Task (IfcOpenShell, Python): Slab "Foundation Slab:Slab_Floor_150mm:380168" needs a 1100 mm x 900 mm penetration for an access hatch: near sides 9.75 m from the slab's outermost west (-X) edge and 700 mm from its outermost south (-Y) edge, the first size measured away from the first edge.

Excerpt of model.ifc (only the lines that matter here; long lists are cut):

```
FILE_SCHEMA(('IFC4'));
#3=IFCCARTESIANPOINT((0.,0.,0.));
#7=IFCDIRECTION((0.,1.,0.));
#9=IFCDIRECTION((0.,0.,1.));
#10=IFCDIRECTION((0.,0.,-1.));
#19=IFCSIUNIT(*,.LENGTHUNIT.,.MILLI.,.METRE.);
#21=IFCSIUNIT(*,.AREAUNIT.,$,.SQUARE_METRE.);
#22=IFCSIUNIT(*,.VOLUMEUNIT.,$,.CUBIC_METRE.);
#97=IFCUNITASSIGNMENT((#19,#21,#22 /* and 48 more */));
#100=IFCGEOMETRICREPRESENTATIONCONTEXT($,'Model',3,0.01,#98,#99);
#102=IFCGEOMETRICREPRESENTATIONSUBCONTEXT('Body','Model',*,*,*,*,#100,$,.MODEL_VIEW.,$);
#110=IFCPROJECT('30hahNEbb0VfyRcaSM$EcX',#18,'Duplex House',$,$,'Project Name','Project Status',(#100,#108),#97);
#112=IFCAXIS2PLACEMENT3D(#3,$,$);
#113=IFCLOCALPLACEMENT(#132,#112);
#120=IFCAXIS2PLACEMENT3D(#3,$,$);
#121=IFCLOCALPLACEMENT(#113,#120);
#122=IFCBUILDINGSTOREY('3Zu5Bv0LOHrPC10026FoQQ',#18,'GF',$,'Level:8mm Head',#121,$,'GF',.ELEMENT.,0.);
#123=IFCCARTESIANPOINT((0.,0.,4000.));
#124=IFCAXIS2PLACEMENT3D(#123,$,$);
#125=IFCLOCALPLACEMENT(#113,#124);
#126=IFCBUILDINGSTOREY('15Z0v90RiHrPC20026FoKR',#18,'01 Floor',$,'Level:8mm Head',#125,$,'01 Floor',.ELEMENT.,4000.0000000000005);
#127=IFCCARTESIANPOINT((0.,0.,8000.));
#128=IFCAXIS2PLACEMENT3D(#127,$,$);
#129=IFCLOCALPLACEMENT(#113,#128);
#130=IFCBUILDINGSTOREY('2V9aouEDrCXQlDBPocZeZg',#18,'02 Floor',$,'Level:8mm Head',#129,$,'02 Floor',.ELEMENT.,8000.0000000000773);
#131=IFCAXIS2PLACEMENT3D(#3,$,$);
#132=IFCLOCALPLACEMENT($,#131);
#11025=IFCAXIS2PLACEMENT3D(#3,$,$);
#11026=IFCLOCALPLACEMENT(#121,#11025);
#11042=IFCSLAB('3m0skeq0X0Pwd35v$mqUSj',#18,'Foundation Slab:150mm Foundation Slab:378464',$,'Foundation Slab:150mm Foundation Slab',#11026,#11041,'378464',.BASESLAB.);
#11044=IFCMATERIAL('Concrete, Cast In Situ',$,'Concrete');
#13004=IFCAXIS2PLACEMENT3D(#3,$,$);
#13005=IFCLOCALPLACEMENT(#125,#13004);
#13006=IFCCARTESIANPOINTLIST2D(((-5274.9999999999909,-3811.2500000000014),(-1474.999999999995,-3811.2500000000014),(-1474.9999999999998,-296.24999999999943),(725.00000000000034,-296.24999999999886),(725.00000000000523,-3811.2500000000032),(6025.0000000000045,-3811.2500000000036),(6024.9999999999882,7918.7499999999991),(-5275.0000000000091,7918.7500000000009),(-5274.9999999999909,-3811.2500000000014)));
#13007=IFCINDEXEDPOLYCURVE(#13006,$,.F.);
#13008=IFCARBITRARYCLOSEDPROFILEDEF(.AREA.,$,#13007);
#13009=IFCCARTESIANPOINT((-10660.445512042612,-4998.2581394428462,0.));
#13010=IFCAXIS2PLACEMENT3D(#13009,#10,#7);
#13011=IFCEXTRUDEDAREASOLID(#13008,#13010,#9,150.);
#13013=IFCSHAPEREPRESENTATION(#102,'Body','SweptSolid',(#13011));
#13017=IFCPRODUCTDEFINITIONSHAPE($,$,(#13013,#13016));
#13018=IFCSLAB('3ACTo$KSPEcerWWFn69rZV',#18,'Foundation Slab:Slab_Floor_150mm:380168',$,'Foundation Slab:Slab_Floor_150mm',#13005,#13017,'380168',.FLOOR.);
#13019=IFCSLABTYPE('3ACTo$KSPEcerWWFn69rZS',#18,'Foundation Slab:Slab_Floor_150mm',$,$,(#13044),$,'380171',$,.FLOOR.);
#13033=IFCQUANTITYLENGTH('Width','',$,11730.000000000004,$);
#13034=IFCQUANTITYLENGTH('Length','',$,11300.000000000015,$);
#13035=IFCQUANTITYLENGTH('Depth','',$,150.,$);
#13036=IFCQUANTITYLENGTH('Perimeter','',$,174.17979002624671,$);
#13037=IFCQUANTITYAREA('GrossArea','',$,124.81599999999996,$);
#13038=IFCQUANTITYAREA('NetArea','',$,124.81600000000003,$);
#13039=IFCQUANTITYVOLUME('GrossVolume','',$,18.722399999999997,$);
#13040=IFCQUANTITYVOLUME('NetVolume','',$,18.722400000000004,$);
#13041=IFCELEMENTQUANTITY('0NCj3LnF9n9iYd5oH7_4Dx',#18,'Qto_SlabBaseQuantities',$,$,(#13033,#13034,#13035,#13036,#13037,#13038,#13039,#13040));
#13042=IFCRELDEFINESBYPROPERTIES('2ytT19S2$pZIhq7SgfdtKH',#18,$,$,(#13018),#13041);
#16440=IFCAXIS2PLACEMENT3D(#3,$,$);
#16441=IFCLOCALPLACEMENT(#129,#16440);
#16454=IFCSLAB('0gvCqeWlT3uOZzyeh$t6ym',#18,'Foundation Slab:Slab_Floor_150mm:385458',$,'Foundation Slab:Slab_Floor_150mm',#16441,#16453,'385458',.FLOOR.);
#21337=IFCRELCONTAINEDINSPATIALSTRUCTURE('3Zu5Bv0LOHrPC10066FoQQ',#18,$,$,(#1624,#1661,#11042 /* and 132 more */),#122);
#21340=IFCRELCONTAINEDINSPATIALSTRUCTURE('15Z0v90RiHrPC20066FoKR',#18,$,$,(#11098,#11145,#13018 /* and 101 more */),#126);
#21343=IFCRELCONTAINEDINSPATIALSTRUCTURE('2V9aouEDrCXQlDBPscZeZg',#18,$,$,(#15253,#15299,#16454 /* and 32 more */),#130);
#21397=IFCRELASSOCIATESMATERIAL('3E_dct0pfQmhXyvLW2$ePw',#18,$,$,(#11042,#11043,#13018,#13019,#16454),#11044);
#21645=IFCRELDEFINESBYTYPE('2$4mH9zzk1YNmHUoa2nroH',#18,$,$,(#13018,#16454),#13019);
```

```python
import numpy as np
import ifcopenshell
import ifcopenshell.api.feature
import ifcopenshell.api.geometry
import ifcopenshell.api.pset
import ifcopenshell.api.root
import ifcopenshell.geom
import ifcopenshell.util.element
import ifcopenshell.util.placement
import ifcopenshell.util.representation
import ifcopenshell.util.shape
import ifcopenshell.util.unit

model = ifcopenshell.open("model.ifc")
unit_scale = ifcopenshell.util.unit.calculate_unit_scale(model)
area_scale = ifcopenshell.util.unit.calculate_unit_scale(model, "AREAUNIT")
volume_scale = ifcopenshell.util.unit.calculate_unit_scale(model, "VOLUMEUNIT")
settings = ifcopenshell.geom.settings()


def volume(element):
    """Net volume in cubic metres, openings subtracted."""
    shape = ifcopenshell.geom.create_shape(settings, element)
    return ifcopenshell.util.shape.get_volume(shape.geometry)


slab = model.by_id(13018)
before = volume(slab)

# Extent in the slab's own axes, in metres. The edges named are its -X and -Y sides.
slab_shape = ifcopenshell.geom.create_shape(settings, slab)
vertices = ifcopenshell.util.shape.get_vertices(slab_shape.geometry)
x_min, y_min, bottom = vertices.min(axis=0)
top = vertices[:, 2].max()

opening = ifcopenshell.api.root.create_entity(model, ifc_class="IfcOpeningElement", name="Access hatch opening", predefined_type="OPENING")
context = ifcopenshell.util.representation.get_context(model, "Model", "Body", "MODEL_VIEW")
width, depth = 1.1, 0.9
outline = [(0.0, 0.0), (width, 0.0), (width, depth), (0.0, depth), (0.0, 0.0)]
# Overshoot both faces by 50 mm so the cut is clean.
shape = ifcopenshell.api.geometry.add_slab_representation(
    model, context=context, depth=top - bottom + 0.1, polyline=outline
)
ifcopenshell.api.geometry.assign_representation(model, product=opening, representation=shape)

matrix = ifcopenshell.util.placement.get_local_placement(slab.ObjectPlacement)
matrix[:, 3] = matrix @ np.append(np.array([x_min + 9.75, y_min + 0.7, bottom - 0.05]) / unit_scale, 1.0)
ifcopenshell.api.geometry.edit_object_placement(model, product=opening, matrix=matrix, is_si=False)
ifcopenshell.api.feature.add_feature(model, feature=opening, element=slab)

after = volume(slab)

# Update the slab's stored quantities.
qto = model.by_id(ifcopenshell.util.element.get_pset(slab, "Qto_SlabBaseQuantities", should_inherit=False)["id"])
ifcopenshell.api.pset.edit_qto(model, qto=qto, properties={
    "NetArea": after / (top - bottom) / area_scale,
    "NetVolume": after / volume_scale,
})

print(f"slab volume {before:.3f} -> {after:.3f} m3")

model.write("model_updated.ifc")
```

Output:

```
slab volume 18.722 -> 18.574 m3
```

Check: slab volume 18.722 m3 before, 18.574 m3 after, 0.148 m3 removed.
